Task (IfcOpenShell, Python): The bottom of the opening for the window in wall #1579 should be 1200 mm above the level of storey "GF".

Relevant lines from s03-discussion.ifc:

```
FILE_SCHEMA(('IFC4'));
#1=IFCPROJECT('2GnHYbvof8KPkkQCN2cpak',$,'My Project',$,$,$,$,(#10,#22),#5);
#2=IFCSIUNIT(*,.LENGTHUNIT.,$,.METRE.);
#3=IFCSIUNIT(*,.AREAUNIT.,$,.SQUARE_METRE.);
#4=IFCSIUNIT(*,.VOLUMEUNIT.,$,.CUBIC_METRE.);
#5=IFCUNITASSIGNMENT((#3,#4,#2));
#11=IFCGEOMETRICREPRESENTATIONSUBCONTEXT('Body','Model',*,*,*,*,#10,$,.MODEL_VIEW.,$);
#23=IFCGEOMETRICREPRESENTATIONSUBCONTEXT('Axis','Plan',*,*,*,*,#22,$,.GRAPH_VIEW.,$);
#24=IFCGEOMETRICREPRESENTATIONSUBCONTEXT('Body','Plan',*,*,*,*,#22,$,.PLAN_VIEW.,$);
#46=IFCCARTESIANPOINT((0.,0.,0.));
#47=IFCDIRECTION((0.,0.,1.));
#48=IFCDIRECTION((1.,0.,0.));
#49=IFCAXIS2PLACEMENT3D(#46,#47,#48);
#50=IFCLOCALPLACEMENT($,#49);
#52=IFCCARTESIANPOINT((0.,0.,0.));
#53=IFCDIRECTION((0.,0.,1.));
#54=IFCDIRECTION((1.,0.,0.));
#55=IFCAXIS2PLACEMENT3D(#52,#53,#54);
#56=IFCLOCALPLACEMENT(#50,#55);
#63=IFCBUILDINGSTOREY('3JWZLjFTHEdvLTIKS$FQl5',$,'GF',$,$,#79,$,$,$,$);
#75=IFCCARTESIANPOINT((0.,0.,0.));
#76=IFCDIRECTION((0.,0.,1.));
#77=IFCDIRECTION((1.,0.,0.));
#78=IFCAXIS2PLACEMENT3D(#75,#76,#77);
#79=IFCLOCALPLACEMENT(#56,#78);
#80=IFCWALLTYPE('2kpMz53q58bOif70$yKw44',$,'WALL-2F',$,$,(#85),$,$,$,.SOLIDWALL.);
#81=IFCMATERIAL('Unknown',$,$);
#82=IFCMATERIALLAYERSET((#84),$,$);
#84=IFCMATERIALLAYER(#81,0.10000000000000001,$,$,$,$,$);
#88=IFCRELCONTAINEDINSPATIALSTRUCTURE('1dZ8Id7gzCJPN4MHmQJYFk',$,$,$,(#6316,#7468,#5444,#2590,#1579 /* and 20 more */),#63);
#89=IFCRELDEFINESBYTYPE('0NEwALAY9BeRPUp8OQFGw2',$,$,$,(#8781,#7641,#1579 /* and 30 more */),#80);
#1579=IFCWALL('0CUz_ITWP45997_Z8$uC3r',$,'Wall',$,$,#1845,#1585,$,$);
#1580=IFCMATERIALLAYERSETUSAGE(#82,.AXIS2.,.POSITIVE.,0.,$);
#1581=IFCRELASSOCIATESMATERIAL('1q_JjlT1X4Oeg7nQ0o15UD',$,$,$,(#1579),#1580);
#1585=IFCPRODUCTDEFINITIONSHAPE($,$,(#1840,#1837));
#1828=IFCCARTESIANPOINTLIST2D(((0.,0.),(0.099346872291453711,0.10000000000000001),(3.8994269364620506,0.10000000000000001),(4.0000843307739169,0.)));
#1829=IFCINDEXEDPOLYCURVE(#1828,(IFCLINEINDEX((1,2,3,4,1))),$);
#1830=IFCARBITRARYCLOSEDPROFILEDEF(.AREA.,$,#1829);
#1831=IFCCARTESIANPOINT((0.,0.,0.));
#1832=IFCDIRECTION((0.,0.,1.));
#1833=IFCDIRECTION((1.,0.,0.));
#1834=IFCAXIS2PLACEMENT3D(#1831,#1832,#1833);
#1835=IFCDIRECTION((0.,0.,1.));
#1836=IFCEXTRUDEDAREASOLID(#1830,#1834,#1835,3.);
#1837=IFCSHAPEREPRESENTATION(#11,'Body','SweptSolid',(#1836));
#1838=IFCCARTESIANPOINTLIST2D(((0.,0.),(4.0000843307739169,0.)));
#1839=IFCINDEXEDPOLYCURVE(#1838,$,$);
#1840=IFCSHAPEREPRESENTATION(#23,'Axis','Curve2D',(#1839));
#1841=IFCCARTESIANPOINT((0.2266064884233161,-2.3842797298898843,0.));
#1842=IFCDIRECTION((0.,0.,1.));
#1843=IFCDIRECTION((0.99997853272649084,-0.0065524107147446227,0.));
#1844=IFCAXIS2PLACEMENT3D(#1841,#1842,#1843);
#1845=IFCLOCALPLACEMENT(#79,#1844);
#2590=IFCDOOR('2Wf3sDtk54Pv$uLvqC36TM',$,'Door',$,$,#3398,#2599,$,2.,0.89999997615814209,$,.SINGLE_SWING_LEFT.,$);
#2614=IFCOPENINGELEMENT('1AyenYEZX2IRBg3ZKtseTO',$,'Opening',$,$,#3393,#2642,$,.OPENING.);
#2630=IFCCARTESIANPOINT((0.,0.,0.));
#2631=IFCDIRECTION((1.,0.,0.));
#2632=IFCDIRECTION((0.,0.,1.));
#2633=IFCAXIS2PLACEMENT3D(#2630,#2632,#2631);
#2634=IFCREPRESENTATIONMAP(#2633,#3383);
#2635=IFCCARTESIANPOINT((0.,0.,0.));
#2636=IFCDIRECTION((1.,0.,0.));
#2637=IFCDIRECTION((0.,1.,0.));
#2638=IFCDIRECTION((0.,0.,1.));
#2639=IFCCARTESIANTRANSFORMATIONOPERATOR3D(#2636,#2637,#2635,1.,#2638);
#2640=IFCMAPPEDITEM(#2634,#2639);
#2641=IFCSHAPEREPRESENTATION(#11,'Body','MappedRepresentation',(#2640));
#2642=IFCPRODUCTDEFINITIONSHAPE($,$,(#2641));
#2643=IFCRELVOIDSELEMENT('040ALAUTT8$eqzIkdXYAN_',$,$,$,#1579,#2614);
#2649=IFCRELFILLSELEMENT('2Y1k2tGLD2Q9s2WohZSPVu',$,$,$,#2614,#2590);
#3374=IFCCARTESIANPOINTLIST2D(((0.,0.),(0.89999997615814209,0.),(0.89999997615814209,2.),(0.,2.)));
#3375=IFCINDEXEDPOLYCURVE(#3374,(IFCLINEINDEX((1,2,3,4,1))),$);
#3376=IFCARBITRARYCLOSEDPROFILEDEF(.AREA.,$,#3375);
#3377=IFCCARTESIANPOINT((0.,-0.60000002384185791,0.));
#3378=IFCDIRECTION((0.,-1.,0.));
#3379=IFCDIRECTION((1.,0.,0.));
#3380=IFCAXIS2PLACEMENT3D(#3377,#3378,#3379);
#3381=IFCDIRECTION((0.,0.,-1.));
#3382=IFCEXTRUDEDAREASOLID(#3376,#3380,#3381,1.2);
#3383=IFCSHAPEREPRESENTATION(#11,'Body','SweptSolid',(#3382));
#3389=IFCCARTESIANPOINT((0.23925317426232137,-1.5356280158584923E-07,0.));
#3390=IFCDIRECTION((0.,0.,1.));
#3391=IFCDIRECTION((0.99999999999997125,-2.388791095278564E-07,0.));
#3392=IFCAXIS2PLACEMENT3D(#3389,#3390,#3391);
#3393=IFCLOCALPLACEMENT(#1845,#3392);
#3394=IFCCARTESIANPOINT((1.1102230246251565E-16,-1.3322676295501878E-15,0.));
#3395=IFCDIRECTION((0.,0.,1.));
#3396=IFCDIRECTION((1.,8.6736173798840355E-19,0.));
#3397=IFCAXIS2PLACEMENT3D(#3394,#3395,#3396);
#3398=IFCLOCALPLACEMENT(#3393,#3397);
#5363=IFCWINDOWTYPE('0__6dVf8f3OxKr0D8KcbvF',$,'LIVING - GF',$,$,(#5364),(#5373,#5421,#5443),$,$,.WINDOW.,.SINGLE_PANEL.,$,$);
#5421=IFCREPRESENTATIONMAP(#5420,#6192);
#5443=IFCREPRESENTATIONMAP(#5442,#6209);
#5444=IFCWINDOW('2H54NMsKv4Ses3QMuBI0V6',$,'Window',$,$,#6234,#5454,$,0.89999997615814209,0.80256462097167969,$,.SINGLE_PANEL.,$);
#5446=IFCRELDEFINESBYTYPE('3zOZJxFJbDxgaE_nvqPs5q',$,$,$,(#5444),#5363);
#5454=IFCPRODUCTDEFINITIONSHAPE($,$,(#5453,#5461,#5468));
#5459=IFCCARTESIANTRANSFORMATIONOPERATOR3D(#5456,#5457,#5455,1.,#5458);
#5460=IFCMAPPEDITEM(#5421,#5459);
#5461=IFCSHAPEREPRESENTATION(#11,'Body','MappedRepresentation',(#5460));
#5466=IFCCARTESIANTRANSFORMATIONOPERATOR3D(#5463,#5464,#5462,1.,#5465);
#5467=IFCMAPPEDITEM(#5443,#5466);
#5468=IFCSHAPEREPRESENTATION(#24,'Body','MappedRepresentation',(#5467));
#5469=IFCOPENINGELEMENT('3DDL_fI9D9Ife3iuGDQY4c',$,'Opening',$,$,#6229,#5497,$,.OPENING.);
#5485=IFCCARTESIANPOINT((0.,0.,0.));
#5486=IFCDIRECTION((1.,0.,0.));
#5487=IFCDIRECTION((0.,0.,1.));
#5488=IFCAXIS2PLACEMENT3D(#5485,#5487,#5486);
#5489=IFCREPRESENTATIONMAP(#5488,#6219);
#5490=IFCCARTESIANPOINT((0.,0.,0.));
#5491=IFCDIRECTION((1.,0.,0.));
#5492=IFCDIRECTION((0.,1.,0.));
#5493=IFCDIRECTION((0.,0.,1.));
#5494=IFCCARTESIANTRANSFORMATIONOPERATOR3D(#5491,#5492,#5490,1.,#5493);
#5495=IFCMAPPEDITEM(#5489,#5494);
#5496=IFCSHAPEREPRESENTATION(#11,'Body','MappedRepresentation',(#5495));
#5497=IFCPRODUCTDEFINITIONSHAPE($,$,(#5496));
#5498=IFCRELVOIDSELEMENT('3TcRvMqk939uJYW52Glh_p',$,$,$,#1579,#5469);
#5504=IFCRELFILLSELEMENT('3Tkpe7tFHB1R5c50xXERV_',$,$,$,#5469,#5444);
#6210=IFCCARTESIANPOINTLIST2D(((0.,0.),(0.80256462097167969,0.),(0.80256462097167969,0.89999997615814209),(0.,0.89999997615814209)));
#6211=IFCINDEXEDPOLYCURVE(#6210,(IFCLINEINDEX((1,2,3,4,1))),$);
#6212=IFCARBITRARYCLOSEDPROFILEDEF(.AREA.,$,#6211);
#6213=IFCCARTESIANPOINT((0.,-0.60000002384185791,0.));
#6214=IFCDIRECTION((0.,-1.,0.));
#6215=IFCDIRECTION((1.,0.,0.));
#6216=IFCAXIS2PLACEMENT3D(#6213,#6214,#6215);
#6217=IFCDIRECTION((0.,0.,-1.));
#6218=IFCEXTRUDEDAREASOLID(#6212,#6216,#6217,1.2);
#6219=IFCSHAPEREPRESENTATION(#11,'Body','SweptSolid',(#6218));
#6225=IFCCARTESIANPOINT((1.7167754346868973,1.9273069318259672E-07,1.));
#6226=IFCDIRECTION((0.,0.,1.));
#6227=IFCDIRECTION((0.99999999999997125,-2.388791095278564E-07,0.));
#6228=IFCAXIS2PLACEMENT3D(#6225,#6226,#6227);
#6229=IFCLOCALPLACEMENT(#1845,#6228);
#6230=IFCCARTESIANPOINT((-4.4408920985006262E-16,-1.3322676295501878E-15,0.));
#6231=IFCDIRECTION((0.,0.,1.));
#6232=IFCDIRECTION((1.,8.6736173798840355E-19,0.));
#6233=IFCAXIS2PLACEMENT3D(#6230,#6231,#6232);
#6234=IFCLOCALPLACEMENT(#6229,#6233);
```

```python
import numpy as np
import ifcopenshell
import ifcopenshell.api.geometry
import ifcopenshell.geom
import ifcopenshell.util.element
import ifcopenshell.util.placement
import ifcopenshell.util.shape
import ifcopenshell.util.unit

model = ifcopenshell.open("s03-discussion.ifc")
unit_scale = ifcopenshell.util.unit.calculate_unit_scale(model)

window = model.by_id(5444)
opening = window.FillsVoids[0].RelatingOpeningElement
storey = ifcopenshell.util.element.get_container(window, ifc_class="IfcBuildingStorey")
level = ifcopenshell.util.placement.get_local_placement(storey.ObjectPlacement)[2, 3]

# The opening's origin need not be at the sill, so measure its lowest point.
shape = ifcopenshell.geom.create_shape(ifcopenshell.geom.settings(), opening)
bottom = ifcopenshell.util.shape.get_shape_bottom_elevation(shape, shape.geometry) / unit_scale
dz = level + 1.2 / unit_scale - bottom

shift = np.array([0.0, 0.0, dz])
# The window is placed relative to its opening, so it follows when the opening moves.
matrix = ifcopenshell.util.placement.get_local_placement(opening.ObjectPlacement)
matrix[:3, 3] += shift
ifcopenshell.api.geometry.edit_object_placement(
    model, product=opening, matrix=matrix, is_si=False, should_transform_children=True
)

print(f"moved by {dz * unit_scale:+.3f} m")

model.write("s03-discussion_edited.ifc")
```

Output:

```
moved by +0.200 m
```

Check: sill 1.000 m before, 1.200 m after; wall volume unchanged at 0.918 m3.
